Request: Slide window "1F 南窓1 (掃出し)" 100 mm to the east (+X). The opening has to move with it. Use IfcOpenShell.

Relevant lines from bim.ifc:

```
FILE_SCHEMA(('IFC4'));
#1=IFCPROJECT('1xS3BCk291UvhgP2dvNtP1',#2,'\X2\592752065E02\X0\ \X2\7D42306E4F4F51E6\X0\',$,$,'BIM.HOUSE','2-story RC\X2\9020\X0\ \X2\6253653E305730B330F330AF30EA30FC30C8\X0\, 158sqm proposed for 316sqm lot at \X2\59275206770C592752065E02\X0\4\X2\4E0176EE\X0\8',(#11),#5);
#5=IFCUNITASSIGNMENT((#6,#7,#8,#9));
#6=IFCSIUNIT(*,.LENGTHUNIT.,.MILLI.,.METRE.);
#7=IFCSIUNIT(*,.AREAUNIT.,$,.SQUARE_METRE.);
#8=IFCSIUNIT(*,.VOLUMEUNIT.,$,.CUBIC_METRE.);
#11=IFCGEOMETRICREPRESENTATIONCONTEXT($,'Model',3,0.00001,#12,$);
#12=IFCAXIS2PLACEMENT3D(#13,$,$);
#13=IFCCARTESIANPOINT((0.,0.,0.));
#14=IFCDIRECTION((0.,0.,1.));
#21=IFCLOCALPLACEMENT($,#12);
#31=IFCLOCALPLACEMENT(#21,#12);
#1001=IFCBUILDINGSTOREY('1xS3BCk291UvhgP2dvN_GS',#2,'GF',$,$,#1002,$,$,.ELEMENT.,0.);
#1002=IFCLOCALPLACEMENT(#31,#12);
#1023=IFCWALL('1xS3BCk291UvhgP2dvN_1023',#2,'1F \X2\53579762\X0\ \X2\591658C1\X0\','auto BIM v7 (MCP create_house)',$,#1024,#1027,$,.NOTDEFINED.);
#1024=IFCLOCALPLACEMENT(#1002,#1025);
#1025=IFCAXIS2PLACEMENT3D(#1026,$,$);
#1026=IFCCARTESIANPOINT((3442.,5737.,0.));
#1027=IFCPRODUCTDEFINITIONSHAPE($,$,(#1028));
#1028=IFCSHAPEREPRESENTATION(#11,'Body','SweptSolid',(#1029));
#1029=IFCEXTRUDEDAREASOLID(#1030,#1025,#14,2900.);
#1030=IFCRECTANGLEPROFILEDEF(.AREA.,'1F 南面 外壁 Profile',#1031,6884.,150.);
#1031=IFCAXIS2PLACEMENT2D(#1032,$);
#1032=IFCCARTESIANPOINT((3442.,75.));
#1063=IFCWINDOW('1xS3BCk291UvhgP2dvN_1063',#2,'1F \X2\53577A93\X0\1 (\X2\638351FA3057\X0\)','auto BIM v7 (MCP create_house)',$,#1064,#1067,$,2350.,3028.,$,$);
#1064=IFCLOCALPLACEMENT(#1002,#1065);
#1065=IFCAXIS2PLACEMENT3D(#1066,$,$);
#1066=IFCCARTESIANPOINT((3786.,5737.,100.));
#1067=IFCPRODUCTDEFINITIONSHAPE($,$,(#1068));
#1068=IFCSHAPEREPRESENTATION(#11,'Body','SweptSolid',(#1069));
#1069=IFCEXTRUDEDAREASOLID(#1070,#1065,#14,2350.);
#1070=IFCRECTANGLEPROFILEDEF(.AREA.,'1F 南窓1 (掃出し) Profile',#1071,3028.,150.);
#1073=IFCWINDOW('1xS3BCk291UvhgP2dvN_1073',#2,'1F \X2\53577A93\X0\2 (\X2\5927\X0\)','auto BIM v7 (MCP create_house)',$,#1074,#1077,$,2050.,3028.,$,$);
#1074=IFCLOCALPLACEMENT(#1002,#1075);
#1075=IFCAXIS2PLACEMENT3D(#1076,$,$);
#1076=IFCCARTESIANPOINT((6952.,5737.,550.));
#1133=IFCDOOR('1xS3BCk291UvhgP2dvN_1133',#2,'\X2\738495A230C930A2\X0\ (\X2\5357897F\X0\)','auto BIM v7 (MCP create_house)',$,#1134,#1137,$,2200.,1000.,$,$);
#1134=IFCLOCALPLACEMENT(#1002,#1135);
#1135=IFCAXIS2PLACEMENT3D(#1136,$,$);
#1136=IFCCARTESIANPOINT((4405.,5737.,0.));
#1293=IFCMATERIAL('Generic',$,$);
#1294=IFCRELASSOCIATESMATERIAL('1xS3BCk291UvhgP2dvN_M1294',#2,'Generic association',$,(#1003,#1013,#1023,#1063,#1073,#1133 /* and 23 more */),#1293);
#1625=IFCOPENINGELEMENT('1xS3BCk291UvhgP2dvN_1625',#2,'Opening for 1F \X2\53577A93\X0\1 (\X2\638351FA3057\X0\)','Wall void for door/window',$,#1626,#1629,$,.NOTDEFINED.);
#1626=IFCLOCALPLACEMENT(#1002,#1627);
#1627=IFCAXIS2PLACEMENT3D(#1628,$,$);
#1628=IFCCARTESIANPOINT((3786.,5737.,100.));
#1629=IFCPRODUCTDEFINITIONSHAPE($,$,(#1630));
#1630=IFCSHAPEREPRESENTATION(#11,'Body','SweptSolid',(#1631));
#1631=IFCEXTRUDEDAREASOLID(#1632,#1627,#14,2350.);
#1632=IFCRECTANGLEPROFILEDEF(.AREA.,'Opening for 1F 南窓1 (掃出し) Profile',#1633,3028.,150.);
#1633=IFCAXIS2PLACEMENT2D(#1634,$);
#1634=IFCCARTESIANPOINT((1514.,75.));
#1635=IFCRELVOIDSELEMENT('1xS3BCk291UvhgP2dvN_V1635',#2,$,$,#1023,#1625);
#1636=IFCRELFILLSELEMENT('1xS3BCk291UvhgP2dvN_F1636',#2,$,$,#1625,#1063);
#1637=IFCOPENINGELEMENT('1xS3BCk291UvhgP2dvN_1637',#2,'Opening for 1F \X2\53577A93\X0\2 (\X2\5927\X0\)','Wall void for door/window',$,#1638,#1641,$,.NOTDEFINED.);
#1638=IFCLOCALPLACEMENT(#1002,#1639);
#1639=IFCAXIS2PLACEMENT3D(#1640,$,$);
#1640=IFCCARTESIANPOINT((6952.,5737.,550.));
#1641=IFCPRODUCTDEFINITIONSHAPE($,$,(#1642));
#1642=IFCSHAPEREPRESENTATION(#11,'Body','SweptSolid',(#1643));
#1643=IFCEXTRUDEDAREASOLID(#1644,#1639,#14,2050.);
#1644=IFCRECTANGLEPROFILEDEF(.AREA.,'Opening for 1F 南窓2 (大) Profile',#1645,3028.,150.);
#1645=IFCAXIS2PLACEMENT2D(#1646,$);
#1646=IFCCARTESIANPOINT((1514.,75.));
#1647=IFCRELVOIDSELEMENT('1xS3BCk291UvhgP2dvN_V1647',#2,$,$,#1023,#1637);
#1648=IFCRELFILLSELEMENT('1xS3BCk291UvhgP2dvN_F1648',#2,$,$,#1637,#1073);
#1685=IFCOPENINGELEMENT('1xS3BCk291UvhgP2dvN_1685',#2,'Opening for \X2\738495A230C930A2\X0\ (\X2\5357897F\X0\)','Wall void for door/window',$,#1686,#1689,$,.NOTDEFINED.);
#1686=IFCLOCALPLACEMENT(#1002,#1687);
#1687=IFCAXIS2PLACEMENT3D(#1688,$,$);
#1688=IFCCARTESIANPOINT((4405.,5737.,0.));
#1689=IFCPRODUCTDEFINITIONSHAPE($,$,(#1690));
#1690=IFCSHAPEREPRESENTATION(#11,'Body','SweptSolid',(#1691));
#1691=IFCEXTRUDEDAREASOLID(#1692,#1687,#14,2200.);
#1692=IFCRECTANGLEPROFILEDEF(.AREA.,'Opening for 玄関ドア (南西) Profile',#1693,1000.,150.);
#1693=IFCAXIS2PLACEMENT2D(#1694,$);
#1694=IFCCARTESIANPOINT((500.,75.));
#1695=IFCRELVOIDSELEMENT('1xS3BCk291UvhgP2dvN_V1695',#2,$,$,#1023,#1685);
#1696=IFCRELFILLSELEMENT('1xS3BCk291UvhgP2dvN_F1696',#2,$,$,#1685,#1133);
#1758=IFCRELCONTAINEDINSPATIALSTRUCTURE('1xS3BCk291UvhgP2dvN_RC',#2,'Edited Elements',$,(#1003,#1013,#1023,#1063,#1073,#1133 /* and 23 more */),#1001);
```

```python
import ifcopenshell
import ifcopenshell.api.geometry
import ifcopenshell.util.placement
import ifcopenshell.util.unit

model = ifcopenshell.open("bim.ifc")
unit_scale = ifcopenshell.util.unit.calculate_unit_scale(model)

window = model.by_id(1063)
opening = window.FillsVoids[0].RelatingOpeningElement
wall = opening.VoidsElements[0].RelatingBuildingElement

wall_matrix = ifcopenshell.util.placement.get_local_placement(wall.ObjectPlacement)
shift = wall_matrix[:3, 0] * 0.1 / unit_scale
before = ifcopenshell.util.placement.get_local_placement(window.ObjectPlacement)[:3, 3].copy()

# The window is not placed relative to its opening, so move both.
for product in (opening, window):
    matrix = ifcopenshell.util.placement.get_local_placement(product.ObjectPlacement)
    matrix[:3, 3] += shift
    ifcopenshell.api.geometry.edit_object_placement(model, product=product, matrix=matrix, is_si=False)

after = ifcopenshell.util.placement.get_local_placement(window.ObjectPlacement)[:3, 3]
print("window moved by", (after - before).round(3) + 0.0)

model.write("bim_v2.ifc")
```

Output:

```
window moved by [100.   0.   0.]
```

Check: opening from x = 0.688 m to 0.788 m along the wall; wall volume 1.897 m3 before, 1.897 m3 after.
